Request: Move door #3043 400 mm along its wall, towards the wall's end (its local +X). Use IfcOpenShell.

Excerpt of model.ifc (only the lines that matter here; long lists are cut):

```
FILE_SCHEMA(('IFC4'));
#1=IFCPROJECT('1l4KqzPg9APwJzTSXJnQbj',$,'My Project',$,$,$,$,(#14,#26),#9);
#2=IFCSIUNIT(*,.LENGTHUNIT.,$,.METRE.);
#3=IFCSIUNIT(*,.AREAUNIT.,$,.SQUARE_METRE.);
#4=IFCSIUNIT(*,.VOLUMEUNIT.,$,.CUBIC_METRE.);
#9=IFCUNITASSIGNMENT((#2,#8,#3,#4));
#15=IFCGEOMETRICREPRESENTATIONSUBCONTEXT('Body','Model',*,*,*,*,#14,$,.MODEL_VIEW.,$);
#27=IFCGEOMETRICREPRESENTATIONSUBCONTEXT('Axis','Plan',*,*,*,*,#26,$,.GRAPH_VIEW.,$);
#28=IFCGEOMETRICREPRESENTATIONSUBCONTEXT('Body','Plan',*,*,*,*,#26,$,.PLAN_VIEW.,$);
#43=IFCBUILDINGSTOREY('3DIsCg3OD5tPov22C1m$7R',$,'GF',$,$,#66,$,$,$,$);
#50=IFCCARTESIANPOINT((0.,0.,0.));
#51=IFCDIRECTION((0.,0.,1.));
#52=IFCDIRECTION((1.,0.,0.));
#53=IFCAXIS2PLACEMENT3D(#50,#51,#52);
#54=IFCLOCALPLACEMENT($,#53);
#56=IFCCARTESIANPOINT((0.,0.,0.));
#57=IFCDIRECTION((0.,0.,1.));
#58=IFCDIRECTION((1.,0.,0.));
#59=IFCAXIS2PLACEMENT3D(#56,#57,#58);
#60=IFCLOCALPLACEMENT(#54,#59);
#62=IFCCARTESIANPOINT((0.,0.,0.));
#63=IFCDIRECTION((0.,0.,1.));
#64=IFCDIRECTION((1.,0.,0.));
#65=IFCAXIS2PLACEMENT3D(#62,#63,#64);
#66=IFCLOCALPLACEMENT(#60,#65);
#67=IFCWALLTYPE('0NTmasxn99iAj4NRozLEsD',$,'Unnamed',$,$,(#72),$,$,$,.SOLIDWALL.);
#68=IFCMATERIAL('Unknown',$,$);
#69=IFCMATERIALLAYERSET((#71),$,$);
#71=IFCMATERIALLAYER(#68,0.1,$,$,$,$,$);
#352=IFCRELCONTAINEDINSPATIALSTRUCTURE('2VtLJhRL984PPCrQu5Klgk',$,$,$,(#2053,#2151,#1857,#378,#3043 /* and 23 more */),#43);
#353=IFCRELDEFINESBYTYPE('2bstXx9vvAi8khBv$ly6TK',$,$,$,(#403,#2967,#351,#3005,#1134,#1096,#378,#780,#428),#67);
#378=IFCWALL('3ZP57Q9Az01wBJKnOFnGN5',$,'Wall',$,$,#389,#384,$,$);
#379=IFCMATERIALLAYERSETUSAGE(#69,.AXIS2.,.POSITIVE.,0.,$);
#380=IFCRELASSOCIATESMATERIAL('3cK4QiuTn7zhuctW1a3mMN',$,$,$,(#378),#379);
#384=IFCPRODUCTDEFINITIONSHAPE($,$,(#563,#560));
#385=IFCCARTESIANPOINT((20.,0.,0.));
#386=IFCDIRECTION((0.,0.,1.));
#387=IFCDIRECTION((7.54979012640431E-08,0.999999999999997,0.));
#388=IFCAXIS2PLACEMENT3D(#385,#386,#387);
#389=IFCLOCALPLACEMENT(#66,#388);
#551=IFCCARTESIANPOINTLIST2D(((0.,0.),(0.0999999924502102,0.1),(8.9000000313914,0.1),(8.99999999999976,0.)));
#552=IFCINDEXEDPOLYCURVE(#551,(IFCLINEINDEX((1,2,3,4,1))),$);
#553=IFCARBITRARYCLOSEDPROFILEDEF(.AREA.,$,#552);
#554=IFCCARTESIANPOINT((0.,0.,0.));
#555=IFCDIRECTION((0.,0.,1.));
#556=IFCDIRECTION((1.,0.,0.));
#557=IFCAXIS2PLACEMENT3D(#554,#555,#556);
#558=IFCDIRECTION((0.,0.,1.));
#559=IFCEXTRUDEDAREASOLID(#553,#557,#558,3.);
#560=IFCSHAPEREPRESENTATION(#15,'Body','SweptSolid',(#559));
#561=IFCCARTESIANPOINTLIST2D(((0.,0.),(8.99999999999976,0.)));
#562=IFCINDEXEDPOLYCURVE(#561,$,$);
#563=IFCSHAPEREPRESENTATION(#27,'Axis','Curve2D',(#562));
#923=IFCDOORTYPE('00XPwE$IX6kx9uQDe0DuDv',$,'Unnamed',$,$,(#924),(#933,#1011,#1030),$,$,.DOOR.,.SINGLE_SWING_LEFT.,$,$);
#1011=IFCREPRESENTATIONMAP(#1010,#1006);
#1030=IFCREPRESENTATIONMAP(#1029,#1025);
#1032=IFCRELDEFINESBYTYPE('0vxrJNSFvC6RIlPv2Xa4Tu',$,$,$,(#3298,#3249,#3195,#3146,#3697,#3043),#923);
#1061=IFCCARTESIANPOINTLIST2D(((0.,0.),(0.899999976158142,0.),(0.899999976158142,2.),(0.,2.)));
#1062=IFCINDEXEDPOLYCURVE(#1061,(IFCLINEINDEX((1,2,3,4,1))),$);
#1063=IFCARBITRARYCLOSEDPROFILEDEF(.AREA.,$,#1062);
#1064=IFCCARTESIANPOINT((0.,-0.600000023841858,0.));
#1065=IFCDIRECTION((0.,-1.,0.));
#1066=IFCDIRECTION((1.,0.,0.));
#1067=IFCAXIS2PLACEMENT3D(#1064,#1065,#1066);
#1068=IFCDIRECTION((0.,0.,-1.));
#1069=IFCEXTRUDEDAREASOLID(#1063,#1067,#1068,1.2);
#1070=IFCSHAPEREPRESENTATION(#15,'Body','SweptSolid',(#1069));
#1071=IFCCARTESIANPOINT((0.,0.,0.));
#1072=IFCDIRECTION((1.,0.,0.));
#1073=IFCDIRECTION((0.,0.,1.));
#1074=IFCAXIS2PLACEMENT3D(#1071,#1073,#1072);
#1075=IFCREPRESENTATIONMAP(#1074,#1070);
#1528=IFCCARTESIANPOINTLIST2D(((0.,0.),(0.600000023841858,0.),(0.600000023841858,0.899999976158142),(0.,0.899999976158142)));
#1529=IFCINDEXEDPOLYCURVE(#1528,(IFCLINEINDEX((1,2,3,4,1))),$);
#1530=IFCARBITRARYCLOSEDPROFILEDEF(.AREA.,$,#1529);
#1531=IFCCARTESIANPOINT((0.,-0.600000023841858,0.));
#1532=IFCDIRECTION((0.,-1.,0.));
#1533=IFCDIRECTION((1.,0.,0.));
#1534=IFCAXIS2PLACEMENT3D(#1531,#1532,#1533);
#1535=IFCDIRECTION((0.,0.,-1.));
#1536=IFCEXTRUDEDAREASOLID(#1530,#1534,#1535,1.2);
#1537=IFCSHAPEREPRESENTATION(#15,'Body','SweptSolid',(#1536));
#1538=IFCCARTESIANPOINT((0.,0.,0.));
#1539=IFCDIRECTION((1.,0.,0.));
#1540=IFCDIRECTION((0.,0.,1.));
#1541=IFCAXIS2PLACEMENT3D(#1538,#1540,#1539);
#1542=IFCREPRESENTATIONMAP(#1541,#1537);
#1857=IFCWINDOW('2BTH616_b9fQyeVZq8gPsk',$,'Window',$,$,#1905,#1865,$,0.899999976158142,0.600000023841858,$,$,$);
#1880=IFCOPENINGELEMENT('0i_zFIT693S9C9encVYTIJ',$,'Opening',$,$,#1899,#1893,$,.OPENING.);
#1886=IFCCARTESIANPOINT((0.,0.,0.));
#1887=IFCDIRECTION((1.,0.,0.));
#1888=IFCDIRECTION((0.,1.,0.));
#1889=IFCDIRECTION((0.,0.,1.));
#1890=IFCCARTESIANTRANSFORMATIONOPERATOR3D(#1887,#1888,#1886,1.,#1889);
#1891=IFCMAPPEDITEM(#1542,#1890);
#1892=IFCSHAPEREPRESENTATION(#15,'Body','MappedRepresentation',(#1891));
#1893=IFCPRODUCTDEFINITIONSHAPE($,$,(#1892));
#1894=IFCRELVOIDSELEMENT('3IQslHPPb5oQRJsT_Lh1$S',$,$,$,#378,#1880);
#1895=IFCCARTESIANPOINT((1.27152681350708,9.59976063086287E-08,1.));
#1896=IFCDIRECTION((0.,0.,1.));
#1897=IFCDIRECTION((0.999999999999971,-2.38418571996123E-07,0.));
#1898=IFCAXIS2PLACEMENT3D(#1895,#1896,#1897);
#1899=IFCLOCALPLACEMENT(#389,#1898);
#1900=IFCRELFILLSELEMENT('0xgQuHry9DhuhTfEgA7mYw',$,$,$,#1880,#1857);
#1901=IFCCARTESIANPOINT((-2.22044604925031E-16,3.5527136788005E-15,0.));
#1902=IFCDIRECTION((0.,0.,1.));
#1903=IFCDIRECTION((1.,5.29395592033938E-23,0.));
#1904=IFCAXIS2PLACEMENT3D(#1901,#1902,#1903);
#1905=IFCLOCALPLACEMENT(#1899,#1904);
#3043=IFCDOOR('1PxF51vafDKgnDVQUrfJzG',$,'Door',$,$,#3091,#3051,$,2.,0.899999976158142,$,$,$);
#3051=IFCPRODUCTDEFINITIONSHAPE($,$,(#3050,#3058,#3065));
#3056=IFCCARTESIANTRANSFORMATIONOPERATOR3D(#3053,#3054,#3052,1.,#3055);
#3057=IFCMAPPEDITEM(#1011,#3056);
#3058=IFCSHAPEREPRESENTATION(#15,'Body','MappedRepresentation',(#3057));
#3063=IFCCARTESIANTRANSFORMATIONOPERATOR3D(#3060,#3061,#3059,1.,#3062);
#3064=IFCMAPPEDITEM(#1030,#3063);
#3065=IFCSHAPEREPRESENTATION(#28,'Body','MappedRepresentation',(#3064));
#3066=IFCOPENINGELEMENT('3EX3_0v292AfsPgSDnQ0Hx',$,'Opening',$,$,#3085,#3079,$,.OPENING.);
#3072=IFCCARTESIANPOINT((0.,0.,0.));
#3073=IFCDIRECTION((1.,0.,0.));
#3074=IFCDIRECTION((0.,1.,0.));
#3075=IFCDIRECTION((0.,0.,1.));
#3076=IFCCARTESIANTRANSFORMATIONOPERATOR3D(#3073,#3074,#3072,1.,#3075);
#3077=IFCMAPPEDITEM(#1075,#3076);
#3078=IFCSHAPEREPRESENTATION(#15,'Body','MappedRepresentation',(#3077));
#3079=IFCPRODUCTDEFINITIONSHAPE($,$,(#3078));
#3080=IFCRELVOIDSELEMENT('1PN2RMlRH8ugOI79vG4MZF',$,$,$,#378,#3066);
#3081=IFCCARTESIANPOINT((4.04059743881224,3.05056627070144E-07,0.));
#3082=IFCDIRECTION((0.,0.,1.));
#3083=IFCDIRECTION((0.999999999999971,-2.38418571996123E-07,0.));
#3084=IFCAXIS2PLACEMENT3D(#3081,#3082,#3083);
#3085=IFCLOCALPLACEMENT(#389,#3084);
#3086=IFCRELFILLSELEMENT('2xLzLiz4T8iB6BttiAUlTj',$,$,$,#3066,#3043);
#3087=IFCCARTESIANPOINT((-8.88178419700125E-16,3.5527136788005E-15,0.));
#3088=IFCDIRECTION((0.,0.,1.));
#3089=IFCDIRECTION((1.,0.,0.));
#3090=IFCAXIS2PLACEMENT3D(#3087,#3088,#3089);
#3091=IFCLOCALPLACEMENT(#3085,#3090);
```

```python
import ifcopenshell
import ifcopenshell.api.geometry
import ifcopenshell.util.placement
import ifcopenshell.util.unit

model = ifcopenshell.open("model.ifc")
unit_scale = ifcopenshell.util.unit.calculate_unit_scale(model)

door = model.by_guid("1PxF51vafDKgnDVQUrfJzG")
opening = door.FillsVoids[0].RelatingOpeningElement
wall = opening.VoidsElements[0].RelatingBuildingElement

wall_matrix = ifcopenshell.util.placement.get_local_placement(wall.ObjectPlacement)
shift = wall_matrix[:3, 0] * 0.4 / unit_scale
before = ifcopenshell.util.placement.get_local_placement(door.ObjectPlacement)[:3, 3].copy()

# The door is placed relative to its opening, so it follows when the opening moves.
matrix = ifcopenshell.util.placement.get_local_placement(opening.ObjectPlacement)
matrix[:3, 3] += shift
ifcopenshell.api.geometry.edit_object_placement(
    model, product=opening, matrix=matrix, is_si=False, should_transform_children=True
)

after = ifcopenshell.util.placement.get_local_placement(door.ObjectPlacement)[:3, 3]
print("door moved by", (after - before).round(3) + 0.0)

model.write("model_edited.ifc")
```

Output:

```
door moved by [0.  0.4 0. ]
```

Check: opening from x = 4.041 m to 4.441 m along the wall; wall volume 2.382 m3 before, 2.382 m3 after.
